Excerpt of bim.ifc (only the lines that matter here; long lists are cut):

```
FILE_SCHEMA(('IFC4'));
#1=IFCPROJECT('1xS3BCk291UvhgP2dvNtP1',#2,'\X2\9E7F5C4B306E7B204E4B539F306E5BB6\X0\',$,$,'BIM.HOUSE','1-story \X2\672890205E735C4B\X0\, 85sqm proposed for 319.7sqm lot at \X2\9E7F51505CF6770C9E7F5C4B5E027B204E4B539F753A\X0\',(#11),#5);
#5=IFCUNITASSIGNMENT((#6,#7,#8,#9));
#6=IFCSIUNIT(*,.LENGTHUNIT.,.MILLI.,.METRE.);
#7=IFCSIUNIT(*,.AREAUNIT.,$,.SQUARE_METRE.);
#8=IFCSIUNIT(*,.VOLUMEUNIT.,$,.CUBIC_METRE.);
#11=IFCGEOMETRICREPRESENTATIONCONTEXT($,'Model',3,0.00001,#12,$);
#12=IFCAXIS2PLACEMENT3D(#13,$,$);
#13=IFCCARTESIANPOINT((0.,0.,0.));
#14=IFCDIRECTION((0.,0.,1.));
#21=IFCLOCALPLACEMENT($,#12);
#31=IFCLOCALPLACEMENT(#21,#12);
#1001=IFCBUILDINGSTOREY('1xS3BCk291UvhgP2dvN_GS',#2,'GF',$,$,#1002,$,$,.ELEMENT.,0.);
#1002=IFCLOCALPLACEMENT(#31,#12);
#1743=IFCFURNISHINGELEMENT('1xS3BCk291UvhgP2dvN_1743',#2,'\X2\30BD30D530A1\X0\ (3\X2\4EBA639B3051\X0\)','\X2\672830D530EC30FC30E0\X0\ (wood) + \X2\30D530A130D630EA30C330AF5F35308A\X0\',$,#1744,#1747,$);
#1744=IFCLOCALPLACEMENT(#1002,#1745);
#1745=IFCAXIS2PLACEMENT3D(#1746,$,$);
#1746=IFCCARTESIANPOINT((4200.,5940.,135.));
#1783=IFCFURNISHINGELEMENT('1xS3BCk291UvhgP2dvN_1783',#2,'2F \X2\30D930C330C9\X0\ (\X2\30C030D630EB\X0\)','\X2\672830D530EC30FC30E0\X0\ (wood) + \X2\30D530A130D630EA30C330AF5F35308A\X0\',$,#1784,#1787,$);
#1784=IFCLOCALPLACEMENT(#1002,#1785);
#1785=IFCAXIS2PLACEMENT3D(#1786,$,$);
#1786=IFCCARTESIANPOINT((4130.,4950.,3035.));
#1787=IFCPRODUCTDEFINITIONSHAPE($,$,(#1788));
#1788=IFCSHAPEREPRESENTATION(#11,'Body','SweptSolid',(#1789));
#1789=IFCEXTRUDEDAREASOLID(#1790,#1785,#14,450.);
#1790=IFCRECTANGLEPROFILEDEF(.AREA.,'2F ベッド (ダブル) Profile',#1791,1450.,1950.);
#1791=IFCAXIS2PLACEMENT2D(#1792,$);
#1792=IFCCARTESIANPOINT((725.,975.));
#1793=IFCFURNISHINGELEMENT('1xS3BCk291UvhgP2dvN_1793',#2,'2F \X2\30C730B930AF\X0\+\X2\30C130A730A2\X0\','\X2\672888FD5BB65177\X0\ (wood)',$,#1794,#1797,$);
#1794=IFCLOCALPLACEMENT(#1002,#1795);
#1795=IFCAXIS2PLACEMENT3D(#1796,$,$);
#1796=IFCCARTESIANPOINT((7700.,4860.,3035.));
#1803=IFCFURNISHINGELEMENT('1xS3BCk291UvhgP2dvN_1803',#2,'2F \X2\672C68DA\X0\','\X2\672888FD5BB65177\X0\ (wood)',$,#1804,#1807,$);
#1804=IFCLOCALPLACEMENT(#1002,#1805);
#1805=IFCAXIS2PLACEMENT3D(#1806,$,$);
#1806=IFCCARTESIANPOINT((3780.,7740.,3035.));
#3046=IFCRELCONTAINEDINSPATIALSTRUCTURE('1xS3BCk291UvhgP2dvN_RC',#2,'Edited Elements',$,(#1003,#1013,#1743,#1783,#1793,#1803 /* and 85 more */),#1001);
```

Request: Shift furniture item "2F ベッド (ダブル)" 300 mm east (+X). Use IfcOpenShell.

```python
import ifcopenshell
import ifcopenshell.api.geometry
import ifcopenshell.util.placement

model = ifcopenshell.open("bim.ifc")

item = model.by_guid("1xS3BCk291UvhgP2dvN_1783")
matrix = ifcopenshell.util.placement.get_local_placement(item.ObjectPlacement)
matrix[0, 3] += 300.0
ifcopenshell.api.geometry.edit_object_placement(model, product=item, matrix=matrix, is_si=False)

print(ifcopenshell.util.placement.get_local_placement(item.ObjectPlacement).round(3) + 0.0)

model.write("bim_rev.ifc")
```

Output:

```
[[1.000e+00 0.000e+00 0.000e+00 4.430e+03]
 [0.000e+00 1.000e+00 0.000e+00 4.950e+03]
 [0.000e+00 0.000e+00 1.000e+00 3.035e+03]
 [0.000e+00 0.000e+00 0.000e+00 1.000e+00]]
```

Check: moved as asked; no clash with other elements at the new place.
